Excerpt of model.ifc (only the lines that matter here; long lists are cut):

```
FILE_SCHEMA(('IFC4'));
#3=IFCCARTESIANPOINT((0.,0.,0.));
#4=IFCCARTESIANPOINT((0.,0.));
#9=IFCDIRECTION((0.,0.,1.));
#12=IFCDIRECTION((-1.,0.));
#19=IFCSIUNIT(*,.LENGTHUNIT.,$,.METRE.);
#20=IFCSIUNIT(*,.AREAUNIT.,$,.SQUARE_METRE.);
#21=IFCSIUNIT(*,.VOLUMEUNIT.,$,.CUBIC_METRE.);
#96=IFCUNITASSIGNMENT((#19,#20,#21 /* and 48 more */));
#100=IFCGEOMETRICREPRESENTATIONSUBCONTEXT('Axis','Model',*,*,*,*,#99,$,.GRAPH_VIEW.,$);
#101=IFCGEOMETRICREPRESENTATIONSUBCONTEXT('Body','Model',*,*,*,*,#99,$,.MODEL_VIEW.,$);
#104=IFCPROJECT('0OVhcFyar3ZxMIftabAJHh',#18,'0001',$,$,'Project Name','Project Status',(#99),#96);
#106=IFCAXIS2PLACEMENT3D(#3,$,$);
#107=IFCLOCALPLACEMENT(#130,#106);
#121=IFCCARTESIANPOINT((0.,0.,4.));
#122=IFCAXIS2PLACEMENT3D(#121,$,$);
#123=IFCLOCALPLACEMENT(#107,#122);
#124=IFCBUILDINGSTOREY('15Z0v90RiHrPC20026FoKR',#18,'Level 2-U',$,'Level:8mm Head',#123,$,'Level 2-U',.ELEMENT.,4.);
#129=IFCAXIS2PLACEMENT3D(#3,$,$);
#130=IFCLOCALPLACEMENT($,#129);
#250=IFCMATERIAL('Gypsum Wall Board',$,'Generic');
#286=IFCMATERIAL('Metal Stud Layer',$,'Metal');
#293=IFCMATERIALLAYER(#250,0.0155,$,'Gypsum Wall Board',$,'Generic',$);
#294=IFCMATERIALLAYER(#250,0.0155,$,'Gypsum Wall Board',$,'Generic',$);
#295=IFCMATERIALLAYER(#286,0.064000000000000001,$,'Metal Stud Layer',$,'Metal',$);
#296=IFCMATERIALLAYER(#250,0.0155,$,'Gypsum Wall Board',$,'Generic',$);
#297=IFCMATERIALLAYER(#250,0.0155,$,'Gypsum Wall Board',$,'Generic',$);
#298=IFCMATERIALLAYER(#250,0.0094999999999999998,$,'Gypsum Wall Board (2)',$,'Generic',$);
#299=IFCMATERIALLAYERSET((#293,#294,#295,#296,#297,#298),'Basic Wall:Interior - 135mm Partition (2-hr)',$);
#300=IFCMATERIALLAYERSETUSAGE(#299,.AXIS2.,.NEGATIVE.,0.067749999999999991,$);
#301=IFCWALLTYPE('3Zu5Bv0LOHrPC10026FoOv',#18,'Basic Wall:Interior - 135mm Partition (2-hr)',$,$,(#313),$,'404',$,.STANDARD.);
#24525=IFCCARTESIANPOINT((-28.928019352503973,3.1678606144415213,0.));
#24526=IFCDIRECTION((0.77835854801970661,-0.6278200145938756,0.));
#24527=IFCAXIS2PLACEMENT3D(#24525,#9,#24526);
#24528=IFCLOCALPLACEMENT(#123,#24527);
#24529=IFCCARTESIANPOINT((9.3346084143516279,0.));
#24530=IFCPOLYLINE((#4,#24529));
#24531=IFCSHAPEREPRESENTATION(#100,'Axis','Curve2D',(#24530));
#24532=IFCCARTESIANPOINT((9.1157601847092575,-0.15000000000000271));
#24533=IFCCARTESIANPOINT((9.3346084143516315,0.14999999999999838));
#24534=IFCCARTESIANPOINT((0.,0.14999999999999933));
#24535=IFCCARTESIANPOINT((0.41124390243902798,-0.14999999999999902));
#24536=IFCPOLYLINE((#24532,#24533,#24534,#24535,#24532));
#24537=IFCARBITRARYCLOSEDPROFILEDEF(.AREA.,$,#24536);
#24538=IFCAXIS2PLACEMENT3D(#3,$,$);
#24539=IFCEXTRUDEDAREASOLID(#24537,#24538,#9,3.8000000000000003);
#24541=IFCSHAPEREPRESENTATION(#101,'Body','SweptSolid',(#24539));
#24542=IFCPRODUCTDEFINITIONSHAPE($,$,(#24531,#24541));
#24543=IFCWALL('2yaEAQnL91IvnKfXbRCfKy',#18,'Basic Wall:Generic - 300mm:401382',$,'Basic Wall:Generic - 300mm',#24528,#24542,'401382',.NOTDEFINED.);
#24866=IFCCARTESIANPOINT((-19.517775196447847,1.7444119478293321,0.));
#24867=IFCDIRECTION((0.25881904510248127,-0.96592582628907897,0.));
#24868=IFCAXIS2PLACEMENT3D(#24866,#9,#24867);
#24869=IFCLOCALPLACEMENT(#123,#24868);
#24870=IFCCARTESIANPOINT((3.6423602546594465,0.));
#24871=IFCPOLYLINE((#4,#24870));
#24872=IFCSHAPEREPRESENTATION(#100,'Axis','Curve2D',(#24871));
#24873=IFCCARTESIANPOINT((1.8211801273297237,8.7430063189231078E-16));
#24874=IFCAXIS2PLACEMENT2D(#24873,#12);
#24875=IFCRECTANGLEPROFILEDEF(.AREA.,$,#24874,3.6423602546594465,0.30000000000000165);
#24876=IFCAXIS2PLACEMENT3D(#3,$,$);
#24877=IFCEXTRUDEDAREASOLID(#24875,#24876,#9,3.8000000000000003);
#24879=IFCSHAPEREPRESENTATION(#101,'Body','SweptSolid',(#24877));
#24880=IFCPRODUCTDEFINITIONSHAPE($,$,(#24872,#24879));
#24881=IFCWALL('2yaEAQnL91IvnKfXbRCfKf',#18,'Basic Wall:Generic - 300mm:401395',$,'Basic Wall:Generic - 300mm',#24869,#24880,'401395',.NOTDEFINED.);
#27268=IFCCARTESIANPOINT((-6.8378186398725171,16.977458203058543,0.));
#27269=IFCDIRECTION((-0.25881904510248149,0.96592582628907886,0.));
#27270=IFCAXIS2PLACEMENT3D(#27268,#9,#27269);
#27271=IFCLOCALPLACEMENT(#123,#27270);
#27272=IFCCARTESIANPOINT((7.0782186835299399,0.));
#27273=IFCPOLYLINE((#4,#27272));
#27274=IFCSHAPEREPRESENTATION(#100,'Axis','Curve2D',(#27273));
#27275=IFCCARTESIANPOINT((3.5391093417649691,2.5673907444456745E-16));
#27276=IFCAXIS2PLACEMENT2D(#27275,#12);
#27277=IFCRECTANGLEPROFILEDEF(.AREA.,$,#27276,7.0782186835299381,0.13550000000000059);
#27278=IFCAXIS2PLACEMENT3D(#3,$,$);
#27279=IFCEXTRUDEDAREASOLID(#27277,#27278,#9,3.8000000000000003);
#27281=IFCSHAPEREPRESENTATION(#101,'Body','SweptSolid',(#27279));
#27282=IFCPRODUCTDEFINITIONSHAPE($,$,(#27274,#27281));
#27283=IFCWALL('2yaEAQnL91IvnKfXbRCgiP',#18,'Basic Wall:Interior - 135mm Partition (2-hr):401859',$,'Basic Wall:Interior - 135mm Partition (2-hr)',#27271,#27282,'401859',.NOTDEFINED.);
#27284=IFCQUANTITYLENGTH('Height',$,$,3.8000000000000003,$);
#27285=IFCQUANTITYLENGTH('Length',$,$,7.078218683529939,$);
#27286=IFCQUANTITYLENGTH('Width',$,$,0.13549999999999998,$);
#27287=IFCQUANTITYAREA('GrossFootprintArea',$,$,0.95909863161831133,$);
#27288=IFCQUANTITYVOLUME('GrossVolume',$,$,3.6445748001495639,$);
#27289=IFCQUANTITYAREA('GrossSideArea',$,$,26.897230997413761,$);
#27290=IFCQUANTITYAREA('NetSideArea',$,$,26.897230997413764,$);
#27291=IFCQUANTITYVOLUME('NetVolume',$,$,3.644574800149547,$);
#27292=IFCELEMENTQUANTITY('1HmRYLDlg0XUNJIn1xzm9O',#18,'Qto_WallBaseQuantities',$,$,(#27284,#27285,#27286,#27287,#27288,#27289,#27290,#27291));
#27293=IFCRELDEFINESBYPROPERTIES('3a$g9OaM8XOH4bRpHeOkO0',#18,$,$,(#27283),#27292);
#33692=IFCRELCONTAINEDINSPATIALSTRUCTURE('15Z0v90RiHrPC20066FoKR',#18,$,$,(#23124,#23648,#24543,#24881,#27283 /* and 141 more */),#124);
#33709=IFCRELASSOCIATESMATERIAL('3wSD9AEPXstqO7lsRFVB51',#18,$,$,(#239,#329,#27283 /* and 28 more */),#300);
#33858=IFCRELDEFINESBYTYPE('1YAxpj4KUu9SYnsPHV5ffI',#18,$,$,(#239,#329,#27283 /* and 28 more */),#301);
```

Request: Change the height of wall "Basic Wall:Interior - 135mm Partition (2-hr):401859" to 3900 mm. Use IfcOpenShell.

```python
import ifcopenshell
import ifcopenshell.api.pset
import ifcopenshell.geom
import ifcopenshell.util.element
import ifcopenshell.util.representation
import ifcopenshell.util.shape
import ifcopenshell.util.unit

model = ifcopenshell.open("model.ifc")
unit_scale = ifcopenshell.util.unit.calculate_unit_scale(model)
area_scale = ifcopenshell.util.unit.calculate_unit_scale(model, "AREAUNIT")
volume_scale = ifcopenshell.util.unit.calculate_unit_scale(model, "VOLUMEUNIT")
settings = ifcopenshell.geom.settings()


def volume(element):
    """Net volume in cubic metres, openings subtracted."""
    shape = ifcopenshell.geom.create_shape(settings, element)
    return ifcopenshell.util.shape.get_volume(shape.geometry)


wall = model.by_guid("2yaEAQnL91IvnKfXbRCgiP")
before = volume(wall)

body = ifcopenshell.util.representation.get_representation(wall, "Model", "Body")
solid = body.Items[0]
old_height = solid.Depth
solid.Depth = 3.9 / unit_scale
after = volume(wall)
thickness = 0.1355  # wall thickness in metres

# Update the stored height, areas and volumes.
qto = model.by_id(ifcopenshell.util.element.get_pset(wall, "Qto_WallBaseQuantities", should_inherit=False)["id"])
ifcopenshell.api.pset.edit_qto(model, qto=qto, properties={
    "Height": solid.Depth,
    "GrossVolume": ifcopenshell.util.element.get_pset(wall, "Qto_WallBaseQuantities", "GrossVolume") * solid.Depth / old_height,
    "GrossSideArea": ifcopenshell.util.element.get_pset(wall, "Qto_WallBaseQuantities", "GrossSideArea") * solid.Depth / old_height,
    "NetSideArea": after / thickness / area_scale,
    "NetVolume": after / volume_scale,
})

print(f"height {old_height:g} -> {solid.Depth:g}, volume {before:.3f} -> {after:.3f} m3")

model.write("model-out.ifc")
```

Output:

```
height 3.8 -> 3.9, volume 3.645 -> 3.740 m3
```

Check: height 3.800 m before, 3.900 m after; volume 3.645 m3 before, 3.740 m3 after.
